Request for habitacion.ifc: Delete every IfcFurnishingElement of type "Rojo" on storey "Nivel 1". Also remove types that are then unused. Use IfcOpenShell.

First a look at what the model holds.

```python
import ifcopenshell
import ifcopenshell.util.element

model = ifcopenshell.open("habitacion.ifc")
print(model.schema)
storey = next(s for s in model.by_type("IfcBuildingStorey") if s.Name == "Nivel 1")
furniture = [e for e in ifcopenshell.util.element.get_decomposition(storey) if e.is_a("IfcFurnishingElement")]
seen = {}
for e in furniture:
    element_type = ifcopenshell.util.element.get_type(e)
    name = element_type.Name if element_type not in (None, e) else None
    seen[name] = seen.get(name, 0) + 1
for name, count in sorted(seen.items(), key=str):
    print(count, "x", name)
```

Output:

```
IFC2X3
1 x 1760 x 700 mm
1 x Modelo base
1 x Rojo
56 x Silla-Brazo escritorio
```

```python
import ifcopenshell
import ifcopenshell.api.root
import ifcopenshell.util.element

model = ifcopenshell.open("habitacion.ifc")

storey = next(s for s in model.by_type("IfcBuildingStorey") if s.Name == "Nivel 1")
furniture = [e for e in ifcopenshell.util.element.get_decomposition(storey) if e.is_a("IfcFurnishingElement")]
targets = [e for e in furniture if (t := ifcopenshell.util.element.get_type(e)) not in (None, e) and t.Name == "Rojo"]
types = {ifcopenshell.util.element.get_type(e) for e in targets} - {None, *targets}

for e in targets:
    ifcopenshell.api.root.remove_product(model, product=e)
print(len(targets), "removed")

unused = [t for t in types if not ifcopenshell.util.element.get_types(t)]
for t in unused:
    ifcopenshell.api.root.remove_product(model, product=t)
print(len(unused), "unused types removed")

model.write("habitacion_updated.ifc")
```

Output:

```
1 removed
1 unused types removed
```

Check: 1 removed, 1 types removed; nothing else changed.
